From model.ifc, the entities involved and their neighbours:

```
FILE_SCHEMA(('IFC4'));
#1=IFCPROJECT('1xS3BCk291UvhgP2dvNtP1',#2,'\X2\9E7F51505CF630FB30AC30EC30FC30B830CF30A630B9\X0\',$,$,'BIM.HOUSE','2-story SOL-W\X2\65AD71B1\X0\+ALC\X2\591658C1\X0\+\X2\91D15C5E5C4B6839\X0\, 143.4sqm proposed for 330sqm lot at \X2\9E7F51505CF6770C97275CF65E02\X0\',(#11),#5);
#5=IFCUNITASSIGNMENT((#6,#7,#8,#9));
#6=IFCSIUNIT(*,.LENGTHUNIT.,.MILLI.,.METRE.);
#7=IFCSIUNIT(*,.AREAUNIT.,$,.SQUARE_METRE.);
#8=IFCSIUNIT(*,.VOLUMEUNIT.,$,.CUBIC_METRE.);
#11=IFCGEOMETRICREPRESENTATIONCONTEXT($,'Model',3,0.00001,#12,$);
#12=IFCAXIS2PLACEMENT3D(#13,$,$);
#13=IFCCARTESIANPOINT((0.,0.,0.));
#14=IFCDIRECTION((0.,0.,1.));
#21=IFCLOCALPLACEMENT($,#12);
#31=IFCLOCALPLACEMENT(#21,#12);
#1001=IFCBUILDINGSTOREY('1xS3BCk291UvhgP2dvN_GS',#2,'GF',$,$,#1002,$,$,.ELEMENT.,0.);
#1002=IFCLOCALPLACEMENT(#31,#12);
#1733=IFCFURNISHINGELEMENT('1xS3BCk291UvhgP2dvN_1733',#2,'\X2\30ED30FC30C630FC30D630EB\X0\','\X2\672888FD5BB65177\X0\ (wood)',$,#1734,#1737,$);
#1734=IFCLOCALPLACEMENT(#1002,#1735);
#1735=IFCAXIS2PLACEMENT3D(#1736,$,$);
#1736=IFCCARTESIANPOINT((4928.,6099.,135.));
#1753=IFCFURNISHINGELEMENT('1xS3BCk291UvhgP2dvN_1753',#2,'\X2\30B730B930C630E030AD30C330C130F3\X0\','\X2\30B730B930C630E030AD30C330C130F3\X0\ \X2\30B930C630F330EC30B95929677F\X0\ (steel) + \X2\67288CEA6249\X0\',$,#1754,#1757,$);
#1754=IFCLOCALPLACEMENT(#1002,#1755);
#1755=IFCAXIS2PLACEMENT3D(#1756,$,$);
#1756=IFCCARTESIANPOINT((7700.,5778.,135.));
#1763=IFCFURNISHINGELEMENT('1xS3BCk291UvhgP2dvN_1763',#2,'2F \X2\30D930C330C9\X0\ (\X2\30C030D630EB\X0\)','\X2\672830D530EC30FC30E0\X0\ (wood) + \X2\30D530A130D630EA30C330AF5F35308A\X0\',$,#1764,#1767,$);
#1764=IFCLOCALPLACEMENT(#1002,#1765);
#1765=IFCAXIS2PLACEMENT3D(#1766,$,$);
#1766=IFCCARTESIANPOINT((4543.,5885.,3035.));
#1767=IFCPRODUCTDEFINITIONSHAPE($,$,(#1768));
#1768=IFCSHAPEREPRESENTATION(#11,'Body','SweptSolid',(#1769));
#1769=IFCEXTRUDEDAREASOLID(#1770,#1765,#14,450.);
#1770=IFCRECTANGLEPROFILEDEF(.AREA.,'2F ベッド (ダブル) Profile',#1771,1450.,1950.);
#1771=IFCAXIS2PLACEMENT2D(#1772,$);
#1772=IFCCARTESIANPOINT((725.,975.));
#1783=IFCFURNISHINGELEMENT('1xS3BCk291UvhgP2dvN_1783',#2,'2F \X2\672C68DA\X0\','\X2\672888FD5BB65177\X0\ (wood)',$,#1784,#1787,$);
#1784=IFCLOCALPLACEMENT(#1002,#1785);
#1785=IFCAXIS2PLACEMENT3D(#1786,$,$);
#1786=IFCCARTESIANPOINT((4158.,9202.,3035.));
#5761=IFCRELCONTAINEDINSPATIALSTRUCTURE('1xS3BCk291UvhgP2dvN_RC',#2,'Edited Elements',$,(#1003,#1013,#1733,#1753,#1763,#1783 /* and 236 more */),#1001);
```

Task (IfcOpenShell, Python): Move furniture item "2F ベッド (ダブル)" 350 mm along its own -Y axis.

```python
import ifcopenshell
import ifcopenshell.api.geometry
import ifcopenshell.util.placement

model = ifcopenshell.open("model.ifc")

item = model.by_id(1763)
matrix = ifcopenshell.util.placement.get_local_placement(item.ObjectPlacement)
matrix[:3, 3] -= matrix[:3, 1] * 350.0
ifcopenshell.api.geometry.edit_object_placement(model, product=item, matrix=matrix, is_si=False)

print(ifcopenshell.util.placement.get_local_placement(item.ObjectPlacement).round(3) + 0.0)

model.write("model_updated.ifc")
```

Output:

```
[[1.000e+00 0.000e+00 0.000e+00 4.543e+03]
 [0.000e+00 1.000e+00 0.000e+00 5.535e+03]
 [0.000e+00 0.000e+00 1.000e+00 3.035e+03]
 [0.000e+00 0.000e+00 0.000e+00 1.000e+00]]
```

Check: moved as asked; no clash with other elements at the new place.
